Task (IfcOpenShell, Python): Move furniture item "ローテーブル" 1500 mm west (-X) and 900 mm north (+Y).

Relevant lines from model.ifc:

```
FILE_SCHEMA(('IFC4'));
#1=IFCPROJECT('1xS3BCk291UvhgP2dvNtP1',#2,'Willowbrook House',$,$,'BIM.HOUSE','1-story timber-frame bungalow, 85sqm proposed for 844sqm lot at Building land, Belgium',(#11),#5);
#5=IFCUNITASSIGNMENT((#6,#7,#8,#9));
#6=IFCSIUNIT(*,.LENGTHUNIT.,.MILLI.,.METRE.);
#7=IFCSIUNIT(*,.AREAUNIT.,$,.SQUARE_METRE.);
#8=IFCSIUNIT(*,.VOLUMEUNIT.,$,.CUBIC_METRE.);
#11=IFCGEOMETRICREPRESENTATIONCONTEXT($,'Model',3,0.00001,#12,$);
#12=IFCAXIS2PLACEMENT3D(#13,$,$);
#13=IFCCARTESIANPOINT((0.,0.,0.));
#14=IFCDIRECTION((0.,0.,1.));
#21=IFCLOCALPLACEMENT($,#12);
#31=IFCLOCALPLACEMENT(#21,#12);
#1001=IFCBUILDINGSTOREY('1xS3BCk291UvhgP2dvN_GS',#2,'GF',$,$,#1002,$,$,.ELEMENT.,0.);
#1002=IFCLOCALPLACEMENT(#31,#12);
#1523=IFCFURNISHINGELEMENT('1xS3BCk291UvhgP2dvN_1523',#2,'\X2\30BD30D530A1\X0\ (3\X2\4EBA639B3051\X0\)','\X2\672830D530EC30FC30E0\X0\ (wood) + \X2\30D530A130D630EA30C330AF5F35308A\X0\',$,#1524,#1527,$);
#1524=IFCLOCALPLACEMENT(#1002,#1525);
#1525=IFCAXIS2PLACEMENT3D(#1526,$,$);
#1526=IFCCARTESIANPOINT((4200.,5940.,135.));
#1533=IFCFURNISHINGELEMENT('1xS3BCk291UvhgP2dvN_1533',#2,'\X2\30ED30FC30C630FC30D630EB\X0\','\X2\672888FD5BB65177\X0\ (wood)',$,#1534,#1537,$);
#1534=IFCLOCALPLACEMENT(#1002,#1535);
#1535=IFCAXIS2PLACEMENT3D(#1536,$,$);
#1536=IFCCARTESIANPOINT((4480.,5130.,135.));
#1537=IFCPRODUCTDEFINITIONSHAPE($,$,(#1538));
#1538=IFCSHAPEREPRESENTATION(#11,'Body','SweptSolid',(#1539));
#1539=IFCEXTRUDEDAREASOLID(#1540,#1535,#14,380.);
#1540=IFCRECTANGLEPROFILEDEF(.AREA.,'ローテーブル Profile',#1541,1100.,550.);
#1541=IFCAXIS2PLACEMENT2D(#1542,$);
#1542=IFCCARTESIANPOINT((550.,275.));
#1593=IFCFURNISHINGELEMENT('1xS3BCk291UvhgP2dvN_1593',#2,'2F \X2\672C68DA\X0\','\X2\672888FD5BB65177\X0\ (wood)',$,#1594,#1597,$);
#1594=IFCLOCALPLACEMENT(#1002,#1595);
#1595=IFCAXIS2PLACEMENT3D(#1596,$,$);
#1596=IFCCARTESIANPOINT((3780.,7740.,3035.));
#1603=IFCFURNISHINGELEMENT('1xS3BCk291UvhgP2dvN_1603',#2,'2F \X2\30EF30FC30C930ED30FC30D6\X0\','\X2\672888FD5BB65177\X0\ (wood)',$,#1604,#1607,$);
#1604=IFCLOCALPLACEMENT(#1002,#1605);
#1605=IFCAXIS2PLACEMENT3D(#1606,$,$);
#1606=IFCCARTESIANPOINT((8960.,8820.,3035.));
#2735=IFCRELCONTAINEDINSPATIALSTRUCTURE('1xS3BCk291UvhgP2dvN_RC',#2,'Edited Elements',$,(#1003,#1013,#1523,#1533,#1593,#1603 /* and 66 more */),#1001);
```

```python
import ifcopenshell
import ifcopenshell.api.geometry
import ifcopenshell.util.placement

model = ifcopenshell.open("model.ifc")

item = model.by_guid("1xS3BCk291UvhgP2dvN_1533")
matrix = ifcopenshell.util.placement.get_local_placement(item.ObjectPlacement)
matrix[0, 3] -= 1500.0
matrix[1, 3] += 900.0
ifcopenshell.api.geometry.edit_object_placement(model, product=item, matrix=matrix, is_si=False)

print(ifcopenshell.util.placement.get_local_placement(item.ObjectPlacement).round(3) + 0.0)

model.write("model-out.ifc")
```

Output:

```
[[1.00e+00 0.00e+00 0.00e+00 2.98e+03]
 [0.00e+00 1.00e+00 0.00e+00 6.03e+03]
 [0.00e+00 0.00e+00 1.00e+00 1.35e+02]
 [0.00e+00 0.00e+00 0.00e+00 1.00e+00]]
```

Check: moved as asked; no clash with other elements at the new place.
